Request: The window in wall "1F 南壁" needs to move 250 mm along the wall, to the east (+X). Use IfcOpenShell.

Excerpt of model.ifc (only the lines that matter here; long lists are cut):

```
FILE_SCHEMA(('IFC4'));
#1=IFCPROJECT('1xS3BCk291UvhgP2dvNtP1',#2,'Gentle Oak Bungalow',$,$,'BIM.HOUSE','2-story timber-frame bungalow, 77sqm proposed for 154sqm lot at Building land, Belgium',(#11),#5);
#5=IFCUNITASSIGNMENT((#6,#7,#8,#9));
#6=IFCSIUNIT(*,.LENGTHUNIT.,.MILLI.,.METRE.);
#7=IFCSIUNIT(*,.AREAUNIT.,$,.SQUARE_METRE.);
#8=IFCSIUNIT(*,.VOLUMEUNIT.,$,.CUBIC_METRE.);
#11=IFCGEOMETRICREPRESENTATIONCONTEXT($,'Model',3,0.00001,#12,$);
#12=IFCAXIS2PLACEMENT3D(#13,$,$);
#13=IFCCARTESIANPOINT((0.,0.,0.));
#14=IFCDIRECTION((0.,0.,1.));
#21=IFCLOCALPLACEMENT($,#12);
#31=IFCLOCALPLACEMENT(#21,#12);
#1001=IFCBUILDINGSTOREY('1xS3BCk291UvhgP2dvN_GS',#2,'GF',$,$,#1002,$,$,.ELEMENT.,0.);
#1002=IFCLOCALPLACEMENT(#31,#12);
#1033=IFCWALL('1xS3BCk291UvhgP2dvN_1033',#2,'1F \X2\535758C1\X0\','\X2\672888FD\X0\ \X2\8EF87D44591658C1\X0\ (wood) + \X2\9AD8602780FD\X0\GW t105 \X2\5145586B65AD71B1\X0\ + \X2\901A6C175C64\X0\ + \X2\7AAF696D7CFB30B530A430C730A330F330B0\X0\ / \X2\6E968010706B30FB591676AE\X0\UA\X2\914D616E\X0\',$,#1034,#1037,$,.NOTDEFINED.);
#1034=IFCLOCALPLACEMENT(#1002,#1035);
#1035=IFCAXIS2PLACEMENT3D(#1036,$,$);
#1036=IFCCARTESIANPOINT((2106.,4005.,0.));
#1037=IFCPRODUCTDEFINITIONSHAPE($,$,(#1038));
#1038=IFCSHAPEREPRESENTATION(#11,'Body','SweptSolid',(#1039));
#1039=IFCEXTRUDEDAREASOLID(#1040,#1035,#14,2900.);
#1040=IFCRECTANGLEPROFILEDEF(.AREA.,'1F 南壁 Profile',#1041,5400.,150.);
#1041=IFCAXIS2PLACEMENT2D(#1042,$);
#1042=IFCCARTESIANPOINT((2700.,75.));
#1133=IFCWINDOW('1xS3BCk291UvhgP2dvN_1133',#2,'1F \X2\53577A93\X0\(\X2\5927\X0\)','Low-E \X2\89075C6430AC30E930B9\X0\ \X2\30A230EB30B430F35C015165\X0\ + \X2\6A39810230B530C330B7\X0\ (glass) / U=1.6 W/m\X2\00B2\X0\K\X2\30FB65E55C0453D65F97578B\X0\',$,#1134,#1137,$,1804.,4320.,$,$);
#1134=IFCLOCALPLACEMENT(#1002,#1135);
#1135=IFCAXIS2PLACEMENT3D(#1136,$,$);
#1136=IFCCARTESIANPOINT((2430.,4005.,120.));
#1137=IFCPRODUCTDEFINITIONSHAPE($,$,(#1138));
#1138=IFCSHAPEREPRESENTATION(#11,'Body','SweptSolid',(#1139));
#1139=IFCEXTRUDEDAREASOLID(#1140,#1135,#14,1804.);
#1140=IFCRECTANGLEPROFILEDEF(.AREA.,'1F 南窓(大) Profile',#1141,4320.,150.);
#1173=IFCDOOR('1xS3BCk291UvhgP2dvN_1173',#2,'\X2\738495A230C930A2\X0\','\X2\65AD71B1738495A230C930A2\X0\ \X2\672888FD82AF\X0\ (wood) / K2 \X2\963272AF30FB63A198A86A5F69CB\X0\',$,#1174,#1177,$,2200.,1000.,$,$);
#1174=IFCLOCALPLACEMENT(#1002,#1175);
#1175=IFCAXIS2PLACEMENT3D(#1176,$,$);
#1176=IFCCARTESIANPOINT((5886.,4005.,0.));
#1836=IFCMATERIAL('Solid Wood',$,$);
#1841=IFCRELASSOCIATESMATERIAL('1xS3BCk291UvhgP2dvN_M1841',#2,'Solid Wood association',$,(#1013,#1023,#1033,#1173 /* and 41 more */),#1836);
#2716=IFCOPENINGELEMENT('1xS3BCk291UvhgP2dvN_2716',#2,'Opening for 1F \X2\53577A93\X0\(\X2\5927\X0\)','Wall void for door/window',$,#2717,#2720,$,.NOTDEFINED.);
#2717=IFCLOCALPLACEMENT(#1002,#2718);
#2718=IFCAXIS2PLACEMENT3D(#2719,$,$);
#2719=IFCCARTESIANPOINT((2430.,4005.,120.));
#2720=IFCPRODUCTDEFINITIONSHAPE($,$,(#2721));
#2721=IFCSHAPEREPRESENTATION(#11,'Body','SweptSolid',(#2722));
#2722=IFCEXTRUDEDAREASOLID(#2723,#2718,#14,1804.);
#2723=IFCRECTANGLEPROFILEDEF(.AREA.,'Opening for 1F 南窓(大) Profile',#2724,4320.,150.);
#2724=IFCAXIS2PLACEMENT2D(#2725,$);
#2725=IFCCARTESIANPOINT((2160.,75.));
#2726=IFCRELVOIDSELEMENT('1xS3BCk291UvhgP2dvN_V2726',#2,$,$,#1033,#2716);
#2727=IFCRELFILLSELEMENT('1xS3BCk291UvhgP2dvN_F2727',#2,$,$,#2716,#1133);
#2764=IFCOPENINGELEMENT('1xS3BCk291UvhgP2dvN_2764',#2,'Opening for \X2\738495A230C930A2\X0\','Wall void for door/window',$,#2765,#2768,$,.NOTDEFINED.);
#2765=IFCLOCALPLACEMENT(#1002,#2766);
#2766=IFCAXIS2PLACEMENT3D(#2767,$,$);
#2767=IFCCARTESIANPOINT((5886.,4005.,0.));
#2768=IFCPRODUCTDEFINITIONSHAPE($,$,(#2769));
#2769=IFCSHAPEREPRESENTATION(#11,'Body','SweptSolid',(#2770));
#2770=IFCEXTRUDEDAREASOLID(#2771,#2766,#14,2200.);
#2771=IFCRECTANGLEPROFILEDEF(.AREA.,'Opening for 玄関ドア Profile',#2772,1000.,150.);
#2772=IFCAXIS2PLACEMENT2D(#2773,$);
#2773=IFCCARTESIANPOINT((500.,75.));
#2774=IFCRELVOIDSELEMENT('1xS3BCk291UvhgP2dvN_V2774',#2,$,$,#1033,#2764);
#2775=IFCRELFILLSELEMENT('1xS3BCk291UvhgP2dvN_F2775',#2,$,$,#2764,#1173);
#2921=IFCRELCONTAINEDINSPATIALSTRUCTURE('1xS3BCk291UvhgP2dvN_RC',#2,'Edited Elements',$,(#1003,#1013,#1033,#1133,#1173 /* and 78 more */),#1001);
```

```python
import ifcopenshell
import ifcopenshell.api.geometry
import ifcopenshell.util.placement
import ifcopenshell.util.unit

model = ifcopenshell.open("model.ifc")
unit_scale = ifcopenshell.util.unit.calculate_unit_scale(model)

window = model.by_id(1133)
opening = window.FillsVoids[0].RelatingOpeningElement
wall = opening.VoidsElements[0].RelatingBuildingElement

wall_matrix = ifcopenshell.util.placement.get_local_placement(wall.ObjectPlacement)
shift = wall_matrix[:3, 0] * 0.25 / unit_scale
before = ifcopenshell.util.placement.get_local_placement(window.ObjectPlacement)[:3, 3].copy()

# The window is not placed relative to its opening, so move both.
for product in (opening, window):
    matrix = ifcopenshell.util.placement.get_local_placement(product.ObjectPlacement)
    matrix[:3, 3] += shift
    ifcopenshell.api.geometry.edit_object_placement(model, product=product, matrix=matrix, is_si=False)

after = ifcopenshell.util.placement.get_local_placement(window.ObjectPlacement)[:3, 3]
print("window moved by", (after - before).round(3) + 0.0)

model.write("model_updated.ifc")
```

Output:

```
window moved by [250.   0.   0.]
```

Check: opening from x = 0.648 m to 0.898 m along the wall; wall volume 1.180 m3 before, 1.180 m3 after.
